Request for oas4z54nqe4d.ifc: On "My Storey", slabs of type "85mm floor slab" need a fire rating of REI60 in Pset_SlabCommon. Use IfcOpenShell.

First a look at what the model holds.

```python
import ifcopenshell
import ifcopenshell.util.element

model = ifcopenshell.open("oas4z54nqe4d.ifc")
print(model.schema)
storey = next(s for s in model.by_type("IfcBuildingStorey") if s.Name == "My Storey")
slabs = [e for e in ifcopenshell.util.element.get_decomposition(storey) if e.is_a("IfcSlab")]
seen = {}
for e in slabs:
    element_type = ifcopenshell.util.element.get_type(e)
    key = (element_type.Name if element_type != e and element_type else None, ifcopenshell.util.element.get_pset(e, "Pset_SlabCommon", "FireRating"))
    seen[key] = seen.get(key, 0) + 1
for (name, value), count in sorted(seen.items(), key=str):
    print(count, "x", name, "|", value)
```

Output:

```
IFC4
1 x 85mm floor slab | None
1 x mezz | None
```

```python
import ifcopenshell
import ifcopenshell.api.pset
import ifcopenshell.util.element

model = ifcopenshell.open("oas4z54nqe4d.ifc")

storey = next(s for s in model.by_type("IfcBuildingStorey") if s.Name == "My Storey")
slabs = [e for e in ifcopenshell.util.element.get_decomposition(storey) if e.is_a("IfcSlab")]

count = 0
for e in slabs:
    element_type = ifcopenshell.util.element.get_type(e)
    if element_type in (None, e) or element_type.Name != "85mm floor slab":
        continue
    # add_pset returns the element's existing set when there is one.
    pset = ifcopenshell.api.pset.add_pset(model, product=e, name="Pset_SlabCommon")
    ifcopenshell.api.pset.edit_pset(model, pset=pset, properties={"FireRating": "REI60"})
    count += 1

print(count, "slabs updated")

model.write("oas4z54nqe4d-out.ifc")
```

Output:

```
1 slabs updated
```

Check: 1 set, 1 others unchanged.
